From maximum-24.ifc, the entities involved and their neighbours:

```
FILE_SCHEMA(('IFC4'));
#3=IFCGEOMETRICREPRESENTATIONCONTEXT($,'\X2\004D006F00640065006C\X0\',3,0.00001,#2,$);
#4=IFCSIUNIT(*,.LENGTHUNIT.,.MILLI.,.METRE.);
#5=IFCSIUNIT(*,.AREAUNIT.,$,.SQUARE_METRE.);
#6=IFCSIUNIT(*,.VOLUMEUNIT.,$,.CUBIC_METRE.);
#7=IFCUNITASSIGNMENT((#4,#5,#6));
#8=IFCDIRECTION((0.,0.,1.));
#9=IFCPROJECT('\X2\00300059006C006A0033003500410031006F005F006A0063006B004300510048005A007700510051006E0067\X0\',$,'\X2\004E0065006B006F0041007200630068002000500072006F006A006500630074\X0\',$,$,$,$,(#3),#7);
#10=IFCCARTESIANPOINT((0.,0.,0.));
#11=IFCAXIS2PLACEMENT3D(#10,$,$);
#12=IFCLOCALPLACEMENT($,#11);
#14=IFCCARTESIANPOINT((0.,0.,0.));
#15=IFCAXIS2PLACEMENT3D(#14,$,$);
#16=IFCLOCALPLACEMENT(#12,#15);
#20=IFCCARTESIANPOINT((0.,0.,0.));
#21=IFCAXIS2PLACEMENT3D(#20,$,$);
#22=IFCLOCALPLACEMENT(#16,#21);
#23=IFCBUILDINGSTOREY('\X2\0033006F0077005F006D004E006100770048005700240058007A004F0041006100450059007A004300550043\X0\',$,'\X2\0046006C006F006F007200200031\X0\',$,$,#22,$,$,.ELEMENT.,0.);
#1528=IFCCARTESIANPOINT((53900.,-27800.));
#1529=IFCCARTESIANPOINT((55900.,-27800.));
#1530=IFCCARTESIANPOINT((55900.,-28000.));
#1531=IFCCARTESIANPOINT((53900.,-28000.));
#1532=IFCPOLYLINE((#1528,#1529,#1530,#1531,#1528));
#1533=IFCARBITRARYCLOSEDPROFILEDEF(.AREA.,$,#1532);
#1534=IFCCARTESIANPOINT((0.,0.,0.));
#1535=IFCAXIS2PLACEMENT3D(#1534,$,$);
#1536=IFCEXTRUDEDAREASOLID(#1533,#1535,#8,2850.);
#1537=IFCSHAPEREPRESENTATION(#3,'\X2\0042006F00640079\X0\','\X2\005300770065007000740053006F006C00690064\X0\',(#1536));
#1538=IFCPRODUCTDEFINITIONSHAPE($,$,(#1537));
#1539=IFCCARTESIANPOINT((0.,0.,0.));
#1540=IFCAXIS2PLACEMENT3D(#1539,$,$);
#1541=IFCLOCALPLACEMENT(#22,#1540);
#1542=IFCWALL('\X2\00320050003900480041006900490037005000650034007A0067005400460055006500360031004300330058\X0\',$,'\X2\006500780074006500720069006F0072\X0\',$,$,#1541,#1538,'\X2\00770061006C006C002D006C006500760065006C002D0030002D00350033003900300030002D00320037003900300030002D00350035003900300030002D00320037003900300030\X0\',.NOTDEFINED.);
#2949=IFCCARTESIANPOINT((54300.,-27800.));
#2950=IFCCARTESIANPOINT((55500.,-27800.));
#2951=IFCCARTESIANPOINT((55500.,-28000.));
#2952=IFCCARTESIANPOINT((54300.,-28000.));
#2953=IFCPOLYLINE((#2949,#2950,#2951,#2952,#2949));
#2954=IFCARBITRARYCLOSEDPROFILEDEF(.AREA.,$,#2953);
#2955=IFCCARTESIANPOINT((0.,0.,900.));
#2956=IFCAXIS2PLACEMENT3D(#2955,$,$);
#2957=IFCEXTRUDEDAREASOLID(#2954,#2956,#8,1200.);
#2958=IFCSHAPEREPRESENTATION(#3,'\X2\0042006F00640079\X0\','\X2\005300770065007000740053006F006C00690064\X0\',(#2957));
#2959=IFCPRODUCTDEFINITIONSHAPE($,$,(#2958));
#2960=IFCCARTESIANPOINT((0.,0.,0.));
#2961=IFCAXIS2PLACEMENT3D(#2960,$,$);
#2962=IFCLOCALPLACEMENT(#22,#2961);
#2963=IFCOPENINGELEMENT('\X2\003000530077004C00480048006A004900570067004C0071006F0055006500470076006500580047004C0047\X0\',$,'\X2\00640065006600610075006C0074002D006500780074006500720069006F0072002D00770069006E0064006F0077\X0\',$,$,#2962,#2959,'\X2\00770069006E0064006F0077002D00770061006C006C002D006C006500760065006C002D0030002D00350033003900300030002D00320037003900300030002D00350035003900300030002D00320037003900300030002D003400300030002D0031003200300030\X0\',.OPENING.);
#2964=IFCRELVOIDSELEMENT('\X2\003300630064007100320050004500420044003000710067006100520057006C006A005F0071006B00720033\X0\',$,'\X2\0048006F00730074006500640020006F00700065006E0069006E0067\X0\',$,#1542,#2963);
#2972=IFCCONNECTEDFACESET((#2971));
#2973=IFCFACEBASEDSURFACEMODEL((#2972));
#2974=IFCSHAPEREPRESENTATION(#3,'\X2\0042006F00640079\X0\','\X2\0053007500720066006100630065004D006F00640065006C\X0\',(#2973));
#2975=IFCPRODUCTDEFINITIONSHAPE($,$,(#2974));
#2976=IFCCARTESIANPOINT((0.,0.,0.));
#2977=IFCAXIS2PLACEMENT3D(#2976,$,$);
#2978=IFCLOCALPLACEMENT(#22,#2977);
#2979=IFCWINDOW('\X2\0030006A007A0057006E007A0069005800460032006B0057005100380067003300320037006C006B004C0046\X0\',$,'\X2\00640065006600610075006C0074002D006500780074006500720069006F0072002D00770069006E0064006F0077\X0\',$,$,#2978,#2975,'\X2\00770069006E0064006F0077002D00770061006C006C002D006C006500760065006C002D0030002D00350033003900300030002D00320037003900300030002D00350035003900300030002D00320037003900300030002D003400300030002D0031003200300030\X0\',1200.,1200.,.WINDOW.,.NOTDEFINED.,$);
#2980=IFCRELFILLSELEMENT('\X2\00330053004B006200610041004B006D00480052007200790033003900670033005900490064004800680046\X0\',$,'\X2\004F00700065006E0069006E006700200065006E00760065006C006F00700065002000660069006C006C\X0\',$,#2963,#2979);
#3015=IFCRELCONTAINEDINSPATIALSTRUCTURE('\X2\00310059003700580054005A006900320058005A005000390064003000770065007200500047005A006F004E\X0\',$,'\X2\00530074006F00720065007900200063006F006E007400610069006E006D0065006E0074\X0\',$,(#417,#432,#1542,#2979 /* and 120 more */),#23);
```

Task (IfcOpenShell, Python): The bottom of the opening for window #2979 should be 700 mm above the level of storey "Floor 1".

```python
import numpy as np
import ifcopenshell
import ifcopenshell.api.geometry
import ifcopenshell.geom
import ifcopenshell.util.element
import ifcopenshell.util.placement
import ifcopenshell.util.shape
import ifcopenshell.util.unit

model = ifcopenshell.open("maximum-24.ifc")
unit_scale = ifcopenshell.util.unit.calculate_unit_scale(model)

window = model.by_guid("0jzWnziXF2kWQ8g327lkLF")
opening = window.FillsVoids[0].RelatingOpeningElement
storey = ifcopenshell.util.element.get_container(window, ifc_class="IfcBuildingStorey")
level = ifcopenshell.util.placement.get_local_placement(storey.ObjectPlacement)[2, 3]

# The opening's origin need not be at the sill, so measure its lowest point.
shape = ifcopenshell.geom.create_shape(ifcopenshell.geom.settings(), opening)
bottom = ifcopenshell.util.shape.get_shape_bottom_elevation(shape, shape.geometry) / unit_scale
dz = level + 700.0 - bottom

shift = np.array([0.0, 0.0, dz])
# The window is not placed relative to its opening, so move both.
for product in (opening, window):
    matrix = ifcopenshell.util.placement.get_local_placement(product.ObjectPlacement)
    matrix[:3, 3] += shift
    ifcopenshell.api.geometry.edit_object_placement(model, product=product, matrix=matrix, is_si=False)

print(f"moved by {dz * unit_scale:+.3f} m")

model.write("maximum-24_rev.ifc")
```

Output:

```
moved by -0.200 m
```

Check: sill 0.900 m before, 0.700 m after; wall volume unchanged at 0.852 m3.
